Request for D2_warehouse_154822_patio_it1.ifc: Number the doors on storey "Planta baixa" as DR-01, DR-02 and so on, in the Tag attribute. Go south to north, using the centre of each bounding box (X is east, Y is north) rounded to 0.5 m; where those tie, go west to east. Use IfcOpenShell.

First a look at what the model holds.

```python
import ifcopenshell
import ifcopenshell.util.element
import ifcopenshell.util.placement

model = ifcopenshell.open("D2_warehouse_154822_patio_it1.ifc")
print(model.schema)
storey = next(s for s in model.by_type("IfcBuildingStorey") if s.Name == "Planta baixa")
doors = [e for e in ifcopenshell.util.element.get_decomposition(storey) if e.is_a("IfcDoor")]
for e in sorted(doors, key=lambda e: e.id()):
    origin = ifcopenshell.util.placement.get_local_placement(e.ObjectPlacement)[:3, 3]
    print(e.id(), e.Tag, e.Name, origin.round(2) + 0.0, sep=" | ")
```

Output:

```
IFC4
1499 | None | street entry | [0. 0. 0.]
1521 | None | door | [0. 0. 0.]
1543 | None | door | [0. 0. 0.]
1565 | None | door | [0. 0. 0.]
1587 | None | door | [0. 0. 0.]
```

```python
import ifcopenshell
import ifcopenshell.geom
import ifcopenshell.util.element
import ifcopenshell.util.shape

model = ifcopenshell.open("D2_warehouse_154822_patio_it1.ifc")
settings = ifcopenshell.geom.settings()
settings.set("use-world-coords", True)


def centre(element):
    shape = ifcopenshell.geom.create_shape(settings, element)
    return ifcopenshell.util.shape.get_bbox_centroid(shape.geometry)


storey = next(s for s in model.by_type("IfcBuildingStorey") if s.Name == "Planta baixa")
doors = [e for e in ifcopenshell.util.element.get_decomposition(storey) if e.is_a("IfcDoor")]

# Insertion points can sit at a corner or the storey origin, so sort by the geometry (in metres).
centres = {e: centre(e) for e in doors}
doors.sort(key=lambda e: (round(centres[e][1] / 0.5), centres[e][0]))

for i, e in enumerate(doors, start=1):
    number = f"DR-{i:02d}"
    e.Tag = number
    print(e.id(), number)

model.write("D2_warehouse_154822_patio_it1_updated.ifc")
```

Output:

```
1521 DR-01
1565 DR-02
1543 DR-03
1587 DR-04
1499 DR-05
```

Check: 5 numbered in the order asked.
